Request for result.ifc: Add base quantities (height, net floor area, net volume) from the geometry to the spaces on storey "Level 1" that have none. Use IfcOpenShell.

First a look at what the model holds.

```python
import ifcopenshell
import ifcopenshell.util.element
import ifcopenshell.util.unit

model = ifcopenshell.open("result.ifc")
print(model.schema)
for unit_type in ("LENGTHUNIT", "AREAUNIT", "VOLUMEUNIT"):
    print(unit_type, ifcopenshell.util.unit.calculate_unit_scale(model, unit_type))
storey = next(s for s in model.by_type("IfcBuildingStorey") if s.Name == "Level 1")
spaces = [e for e in ifcopenshell.util.element.get_decomposition(storey) if e.is_a("IfcSpace")]
for e in sorted(spaces, key=lambda e: e.id()):
    print(e.id(), e.is_a(), e.Name, list(ifcopenshell.util.element.get_psets(e, qtos_only=True)), sep=" | ")
```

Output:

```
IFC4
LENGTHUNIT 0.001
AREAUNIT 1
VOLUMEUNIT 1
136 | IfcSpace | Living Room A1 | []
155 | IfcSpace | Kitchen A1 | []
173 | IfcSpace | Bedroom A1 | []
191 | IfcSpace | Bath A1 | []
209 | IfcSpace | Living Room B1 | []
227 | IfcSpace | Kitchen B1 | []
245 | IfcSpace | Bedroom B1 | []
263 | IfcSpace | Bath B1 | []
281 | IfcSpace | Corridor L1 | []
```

```python
import ifcopenshell
import ifcopenshell.api.pset
import ifcopenshell.geom
import ifcopenshell.util.element
import ifcopenshell.util.shape
import ifcopenshell.util.unit

model = ifcopenshell.open("result.ifc")
unit_scale = ifcopenshell.util.unit.calculate_unit_scale(model)
area_scale = ifcopenshell.util.unit.calculate_unit_scale(model, "AREAUNIT")
volume_scale = ifcopenshell.util.unit.calculate_unit_scale(model, "VOLUMEUNIT")
settings = ifcopenshell.geom.settings()

storey = next(s for s in model.by_type("IfcBuildingStorey") if s.Name == "Level 1")
spaces = [e for e in ifcopenshell.util.element.get_decomposition(storey) if e.is_a("IfcSpace")]

for e in sorted(spaces, key=lambda e: e.id()):
    if ifcopenshell.util.element.get_psets(e, qtos_only=True, should_inherit=False):
        continue
    # Geometry comes back in metres, in the element's own axes.
    shape = ifcopenshell.geom.create_shape(settings, e)
    values = {
        "Height": ifcopenshell.util.shape.get_z(shape.geometry) / unit_scale,
        "NetFloorArea": ifcopenshell.util.shape.get_footprint_area(shape.geometry) / area_scale,
        "NetVolume": ifcopenshell.util.shape.get_volume(shape.geometry) / volume_scale,
    }
    qto = ifcopenshell.api.pset.add_qto(model, product=e, name="Qto_SpaceBaseQuantities")
    ifcopenshell.api.pset.edit_qto(model, qto=qto, properties=values)
    print(e.id(), {k: round(v, 3) for k, v in values.items()})

model.write("result_rev.ifc")
```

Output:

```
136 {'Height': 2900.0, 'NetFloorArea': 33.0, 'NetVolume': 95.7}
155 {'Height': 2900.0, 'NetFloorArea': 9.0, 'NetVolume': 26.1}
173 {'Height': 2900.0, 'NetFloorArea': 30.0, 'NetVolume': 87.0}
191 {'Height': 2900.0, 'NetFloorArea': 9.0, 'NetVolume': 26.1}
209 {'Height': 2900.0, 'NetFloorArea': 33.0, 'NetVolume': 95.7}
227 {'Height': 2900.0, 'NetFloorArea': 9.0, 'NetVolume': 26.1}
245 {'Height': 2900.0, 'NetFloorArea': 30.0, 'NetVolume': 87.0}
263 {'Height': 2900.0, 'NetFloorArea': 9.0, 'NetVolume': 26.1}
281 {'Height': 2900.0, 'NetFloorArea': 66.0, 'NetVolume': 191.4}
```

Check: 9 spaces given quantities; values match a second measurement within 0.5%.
